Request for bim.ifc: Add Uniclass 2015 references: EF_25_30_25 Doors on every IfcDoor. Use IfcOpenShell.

First a look at what the model holds.

```python
import ifcopenshell

model = ifcopenshell.open("bim.ifc")
print(model.schema)
print("classifications:", [c.Name for c in model.by_type("IfcClassification")])
for ifc_class in ("IfcDoor", "IfcRoof", "IfcStair", "IfcWall", "IfcWindow"):
    print(ifc_class, len(model.by_type(ifc_class)))
```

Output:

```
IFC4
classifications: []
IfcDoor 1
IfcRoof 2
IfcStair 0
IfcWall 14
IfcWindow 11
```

```python
import ifcopenshell
import ifcopenshell.api.classification

model = ifcopenshell.open("bim.ifc")

system = ifcopenshell.api.classification.add_classification(model, classification="Uniclass 2015")

codes = {
    "IfcDoor": ("EF_25_30_25", "Doors"),
}
for ifc_class, (code, name) in codes.items():
    products = model.by_type(ifc_class)
    ifcopenshell.api.classification.add_reference(
        model, products=products, classification=system, identification=code, name=name
    )
    print(code, len(products))

model.write("bim_updated.ifc")
```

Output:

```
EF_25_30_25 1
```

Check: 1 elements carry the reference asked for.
